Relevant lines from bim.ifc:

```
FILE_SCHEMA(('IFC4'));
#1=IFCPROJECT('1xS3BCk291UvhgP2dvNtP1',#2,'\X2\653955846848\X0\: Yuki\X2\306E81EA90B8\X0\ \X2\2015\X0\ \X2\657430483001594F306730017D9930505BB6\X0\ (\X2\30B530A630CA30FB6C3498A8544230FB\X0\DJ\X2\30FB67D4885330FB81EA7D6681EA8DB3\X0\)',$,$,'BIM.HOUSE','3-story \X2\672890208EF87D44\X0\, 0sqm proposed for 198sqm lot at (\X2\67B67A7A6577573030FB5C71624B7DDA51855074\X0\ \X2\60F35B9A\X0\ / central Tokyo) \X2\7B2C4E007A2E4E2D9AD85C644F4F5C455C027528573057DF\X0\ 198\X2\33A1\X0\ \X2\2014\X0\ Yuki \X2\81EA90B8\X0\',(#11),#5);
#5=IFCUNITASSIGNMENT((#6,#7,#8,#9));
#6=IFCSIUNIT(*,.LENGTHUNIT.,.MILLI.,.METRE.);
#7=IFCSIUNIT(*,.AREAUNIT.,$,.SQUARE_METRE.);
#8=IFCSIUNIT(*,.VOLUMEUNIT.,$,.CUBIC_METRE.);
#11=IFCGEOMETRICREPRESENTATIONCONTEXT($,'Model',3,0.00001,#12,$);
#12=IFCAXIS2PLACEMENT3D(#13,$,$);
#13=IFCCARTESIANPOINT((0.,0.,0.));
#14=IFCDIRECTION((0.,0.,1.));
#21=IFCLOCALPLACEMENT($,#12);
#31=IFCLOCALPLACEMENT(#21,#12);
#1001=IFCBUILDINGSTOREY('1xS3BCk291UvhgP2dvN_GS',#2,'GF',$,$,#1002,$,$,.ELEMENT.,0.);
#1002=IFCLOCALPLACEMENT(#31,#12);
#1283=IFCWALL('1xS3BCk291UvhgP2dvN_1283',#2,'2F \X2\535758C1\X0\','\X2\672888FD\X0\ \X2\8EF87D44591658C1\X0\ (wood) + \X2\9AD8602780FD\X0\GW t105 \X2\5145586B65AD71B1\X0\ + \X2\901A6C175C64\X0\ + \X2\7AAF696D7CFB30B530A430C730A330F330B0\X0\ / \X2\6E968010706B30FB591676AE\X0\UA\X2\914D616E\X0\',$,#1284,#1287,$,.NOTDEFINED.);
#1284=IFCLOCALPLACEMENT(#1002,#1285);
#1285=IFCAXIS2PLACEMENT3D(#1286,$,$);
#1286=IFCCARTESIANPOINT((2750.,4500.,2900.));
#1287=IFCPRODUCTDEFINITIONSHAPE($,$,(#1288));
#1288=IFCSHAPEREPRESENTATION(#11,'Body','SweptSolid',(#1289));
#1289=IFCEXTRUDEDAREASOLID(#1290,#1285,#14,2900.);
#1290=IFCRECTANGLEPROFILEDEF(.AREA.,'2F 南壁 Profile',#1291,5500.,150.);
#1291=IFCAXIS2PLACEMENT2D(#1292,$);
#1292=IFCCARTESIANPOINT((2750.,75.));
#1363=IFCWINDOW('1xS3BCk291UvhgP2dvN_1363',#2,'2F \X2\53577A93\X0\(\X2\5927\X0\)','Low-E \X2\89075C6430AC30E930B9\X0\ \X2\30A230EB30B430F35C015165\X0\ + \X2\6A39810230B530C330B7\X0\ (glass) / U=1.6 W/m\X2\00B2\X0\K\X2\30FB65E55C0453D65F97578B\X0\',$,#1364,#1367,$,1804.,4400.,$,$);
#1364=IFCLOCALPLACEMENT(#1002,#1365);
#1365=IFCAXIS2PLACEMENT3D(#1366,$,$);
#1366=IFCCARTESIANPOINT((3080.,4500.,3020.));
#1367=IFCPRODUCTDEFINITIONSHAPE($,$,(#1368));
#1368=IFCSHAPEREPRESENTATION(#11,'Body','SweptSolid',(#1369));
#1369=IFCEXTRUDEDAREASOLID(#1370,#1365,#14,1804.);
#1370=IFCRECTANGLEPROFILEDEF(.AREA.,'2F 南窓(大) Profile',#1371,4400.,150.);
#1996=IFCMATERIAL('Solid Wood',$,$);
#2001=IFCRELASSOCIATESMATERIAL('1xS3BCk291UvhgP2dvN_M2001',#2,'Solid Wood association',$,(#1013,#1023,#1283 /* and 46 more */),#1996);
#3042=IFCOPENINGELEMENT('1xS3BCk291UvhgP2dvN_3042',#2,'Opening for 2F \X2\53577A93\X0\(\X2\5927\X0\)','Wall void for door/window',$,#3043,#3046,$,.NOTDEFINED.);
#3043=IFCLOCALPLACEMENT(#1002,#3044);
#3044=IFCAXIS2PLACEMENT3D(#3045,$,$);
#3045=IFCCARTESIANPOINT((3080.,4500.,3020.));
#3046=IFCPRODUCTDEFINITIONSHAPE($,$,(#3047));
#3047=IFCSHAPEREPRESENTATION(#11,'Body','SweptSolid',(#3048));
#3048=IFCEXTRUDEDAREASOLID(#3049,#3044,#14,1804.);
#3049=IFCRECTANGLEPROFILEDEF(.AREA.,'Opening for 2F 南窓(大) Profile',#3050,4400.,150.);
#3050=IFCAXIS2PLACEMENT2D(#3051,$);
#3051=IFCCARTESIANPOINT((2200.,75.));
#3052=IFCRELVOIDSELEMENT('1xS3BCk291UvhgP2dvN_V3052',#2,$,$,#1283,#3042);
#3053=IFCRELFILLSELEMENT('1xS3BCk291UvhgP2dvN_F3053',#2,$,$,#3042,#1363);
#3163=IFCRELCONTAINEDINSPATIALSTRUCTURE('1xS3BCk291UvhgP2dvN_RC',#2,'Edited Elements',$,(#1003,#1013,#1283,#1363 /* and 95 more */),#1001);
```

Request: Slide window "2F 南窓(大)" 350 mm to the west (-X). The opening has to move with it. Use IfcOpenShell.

```python
import ifcopenshell
import ifcopenshell.api.geometry
import ifcopenshell.util.placement
import ifcopenshell.util.unit

model = ifcopenshell.open("bim.ifc")
unit_scale = ifcopenshell.util.unit.calculate_unit_scale(model)

window = model.by_id(1363)
opening = window.FillsVoids[0].RelatingOpeningElement
wall = opening.VoidsElements[0].RelatingBuildingElement

wall_matrix = ifcopenshell.util.placement.get_local_placement(wall.ObjectPlacement)
shift = wall_matrix[:3, 0] * -0.35 / unit_scale
before = ifcopenshell.util.placement.get_local_placement(window.ObjectPlacement)[:3, 3].copy()

# The window is not placed relative to its opening, so move both.
for product in (opening, window):
    matrix = ifcopenshell.util.placement.get_local_placement(product.ObjectPlacement)
    matrix[:3, 3] += shift
    ifcopenshell.api.geometry.edit_object_placement(model, product=product, matrix=matrix, is_si=False)

after = ifcopenshell.util.placement.get_local_placement(window.ObjectPlacement)[:3, 3]
print("window moved by", (after - before).round(3) + 0.0)

model.write("bim_v2.ifc")
```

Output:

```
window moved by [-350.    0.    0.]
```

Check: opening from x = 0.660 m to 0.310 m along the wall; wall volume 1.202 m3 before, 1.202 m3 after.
